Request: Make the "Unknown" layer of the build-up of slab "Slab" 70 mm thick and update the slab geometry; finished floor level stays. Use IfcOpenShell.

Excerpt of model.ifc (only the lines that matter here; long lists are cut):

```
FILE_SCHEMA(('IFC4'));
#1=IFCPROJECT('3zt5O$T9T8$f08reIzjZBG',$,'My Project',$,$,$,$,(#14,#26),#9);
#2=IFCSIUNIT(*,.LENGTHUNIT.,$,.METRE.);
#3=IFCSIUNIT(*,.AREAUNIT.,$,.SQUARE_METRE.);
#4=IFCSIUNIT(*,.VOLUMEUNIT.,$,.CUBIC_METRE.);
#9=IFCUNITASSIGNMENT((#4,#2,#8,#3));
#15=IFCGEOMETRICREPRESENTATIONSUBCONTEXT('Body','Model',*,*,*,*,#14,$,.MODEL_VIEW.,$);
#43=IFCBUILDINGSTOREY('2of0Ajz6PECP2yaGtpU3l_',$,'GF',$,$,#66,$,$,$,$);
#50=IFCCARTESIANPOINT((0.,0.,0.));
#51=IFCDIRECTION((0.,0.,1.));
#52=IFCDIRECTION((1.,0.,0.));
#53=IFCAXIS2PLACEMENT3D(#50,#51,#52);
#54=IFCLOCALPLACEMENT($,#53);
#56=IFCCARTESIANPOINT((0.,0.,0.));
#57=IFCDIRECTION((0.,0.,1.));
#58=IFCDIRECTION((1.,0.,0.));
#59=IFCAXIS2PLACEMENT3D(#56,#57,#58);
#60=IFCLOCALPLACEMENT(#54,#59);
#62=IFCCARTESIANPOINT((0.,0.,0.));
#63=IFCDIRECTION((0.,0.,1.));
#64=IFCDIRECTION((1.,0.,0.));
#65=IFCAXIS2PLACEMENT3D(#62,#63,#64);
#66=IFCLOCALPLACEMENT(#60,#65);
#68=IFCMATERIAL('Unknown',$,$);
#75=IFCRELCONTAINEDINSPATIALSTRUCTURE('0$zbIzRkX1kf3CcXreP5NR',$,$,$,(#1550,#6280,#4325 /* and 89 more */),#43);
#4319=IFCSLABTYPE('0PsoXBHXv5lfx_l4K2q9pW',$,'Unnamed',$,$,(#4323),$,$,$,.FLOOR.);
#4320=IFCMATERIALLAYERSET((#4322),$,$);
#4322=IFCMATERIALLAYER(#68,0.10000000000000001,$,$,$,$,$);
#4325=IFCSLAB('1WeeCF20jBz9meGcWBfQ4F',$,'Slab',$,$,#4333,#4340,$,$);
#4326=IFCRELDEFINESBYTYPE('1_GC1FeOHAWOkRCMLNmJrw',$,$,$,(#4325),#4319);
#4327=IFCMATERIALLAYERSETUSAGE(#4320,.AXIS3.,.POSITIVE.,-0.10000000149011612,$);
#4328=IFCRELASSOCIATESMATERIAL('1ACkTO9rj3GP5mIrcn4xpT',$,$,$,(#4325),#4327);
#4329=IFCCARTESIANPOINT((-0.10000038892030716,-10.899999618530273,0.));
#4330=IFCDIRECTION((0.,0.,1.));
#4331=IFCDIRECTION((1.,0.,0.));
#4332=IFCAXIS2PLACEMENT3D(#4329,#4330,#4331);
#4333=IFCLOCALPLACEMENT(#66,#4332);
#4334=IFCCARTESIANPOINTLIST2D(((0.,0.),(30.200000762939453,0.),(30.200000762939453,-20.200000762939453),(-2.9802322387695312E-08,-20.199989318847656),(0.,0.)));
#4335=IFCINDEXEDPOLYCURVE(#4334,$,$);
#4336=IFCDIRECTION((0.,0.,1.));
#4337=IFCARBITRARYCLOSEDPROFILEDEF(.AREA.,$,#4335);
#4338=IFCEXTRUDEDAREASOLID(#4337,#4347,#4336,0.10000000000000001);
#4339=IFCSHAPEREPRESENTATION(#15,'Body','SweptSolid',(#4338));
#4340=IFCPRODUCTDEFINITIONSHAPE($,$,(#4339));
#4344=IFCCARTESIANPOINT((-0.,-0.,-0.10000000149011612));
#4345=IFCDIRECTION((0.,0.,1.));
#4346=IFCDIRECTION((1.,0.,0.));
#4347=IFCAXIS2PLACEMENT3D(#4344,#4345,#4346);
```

```python
import ifcopenshell
import ifcopenshell.util.element
import ifcopenshell.util.representation
import ifcopenshell.util.unit

model = ifcopenshell.open("model.ifc")
unit_scale = ifcopenshell.util.unit.calculate_unit_scale(model)

layer_set = model.by_id(4320)
layer = next(l for l in layer_set.MaterialLayers if l.Material and l.Material.Name == "Unknown")
change = 0.07 / unit_scale - layer.LayerThickness
layer.LayerThickness += change

# Geometry does not follow the layer set by itself.
slabs = [e for e in ifcopenshell.util.element.get_elements_by_material(model, layer_set) if e.is_a("IfcSlab")]
for slab in sorted(slabs, key=lambda e: e.id()):
    body = ifcopenshell.util.representation.get_representation(slab, "Model", "Body")
    solid = body.Items[0]
    old_depth = solid.Depth
    solid.Depth += change
    # Extruded upwards: lower the start of the extrusion so the top stays.
    x, y, z = solid.Position.Location.Coordinates
    solid.Position.Location = model.createIfcCartesianPoint((x, y, z - change))
    print(slab.id(), f"{old_depth:g} -> {solid.Depth:g}")

# The layers are counted up from the underside, which has moved.
for usage in {ifcopenshell.util.element.get_material(slab) for slab in slabs}:
    usage.OffsetFromReferenceLine -= change

model.write("model_updated.ifc")
```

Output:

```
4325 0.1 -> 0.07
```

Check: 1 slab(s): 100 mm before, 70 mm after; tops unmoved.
